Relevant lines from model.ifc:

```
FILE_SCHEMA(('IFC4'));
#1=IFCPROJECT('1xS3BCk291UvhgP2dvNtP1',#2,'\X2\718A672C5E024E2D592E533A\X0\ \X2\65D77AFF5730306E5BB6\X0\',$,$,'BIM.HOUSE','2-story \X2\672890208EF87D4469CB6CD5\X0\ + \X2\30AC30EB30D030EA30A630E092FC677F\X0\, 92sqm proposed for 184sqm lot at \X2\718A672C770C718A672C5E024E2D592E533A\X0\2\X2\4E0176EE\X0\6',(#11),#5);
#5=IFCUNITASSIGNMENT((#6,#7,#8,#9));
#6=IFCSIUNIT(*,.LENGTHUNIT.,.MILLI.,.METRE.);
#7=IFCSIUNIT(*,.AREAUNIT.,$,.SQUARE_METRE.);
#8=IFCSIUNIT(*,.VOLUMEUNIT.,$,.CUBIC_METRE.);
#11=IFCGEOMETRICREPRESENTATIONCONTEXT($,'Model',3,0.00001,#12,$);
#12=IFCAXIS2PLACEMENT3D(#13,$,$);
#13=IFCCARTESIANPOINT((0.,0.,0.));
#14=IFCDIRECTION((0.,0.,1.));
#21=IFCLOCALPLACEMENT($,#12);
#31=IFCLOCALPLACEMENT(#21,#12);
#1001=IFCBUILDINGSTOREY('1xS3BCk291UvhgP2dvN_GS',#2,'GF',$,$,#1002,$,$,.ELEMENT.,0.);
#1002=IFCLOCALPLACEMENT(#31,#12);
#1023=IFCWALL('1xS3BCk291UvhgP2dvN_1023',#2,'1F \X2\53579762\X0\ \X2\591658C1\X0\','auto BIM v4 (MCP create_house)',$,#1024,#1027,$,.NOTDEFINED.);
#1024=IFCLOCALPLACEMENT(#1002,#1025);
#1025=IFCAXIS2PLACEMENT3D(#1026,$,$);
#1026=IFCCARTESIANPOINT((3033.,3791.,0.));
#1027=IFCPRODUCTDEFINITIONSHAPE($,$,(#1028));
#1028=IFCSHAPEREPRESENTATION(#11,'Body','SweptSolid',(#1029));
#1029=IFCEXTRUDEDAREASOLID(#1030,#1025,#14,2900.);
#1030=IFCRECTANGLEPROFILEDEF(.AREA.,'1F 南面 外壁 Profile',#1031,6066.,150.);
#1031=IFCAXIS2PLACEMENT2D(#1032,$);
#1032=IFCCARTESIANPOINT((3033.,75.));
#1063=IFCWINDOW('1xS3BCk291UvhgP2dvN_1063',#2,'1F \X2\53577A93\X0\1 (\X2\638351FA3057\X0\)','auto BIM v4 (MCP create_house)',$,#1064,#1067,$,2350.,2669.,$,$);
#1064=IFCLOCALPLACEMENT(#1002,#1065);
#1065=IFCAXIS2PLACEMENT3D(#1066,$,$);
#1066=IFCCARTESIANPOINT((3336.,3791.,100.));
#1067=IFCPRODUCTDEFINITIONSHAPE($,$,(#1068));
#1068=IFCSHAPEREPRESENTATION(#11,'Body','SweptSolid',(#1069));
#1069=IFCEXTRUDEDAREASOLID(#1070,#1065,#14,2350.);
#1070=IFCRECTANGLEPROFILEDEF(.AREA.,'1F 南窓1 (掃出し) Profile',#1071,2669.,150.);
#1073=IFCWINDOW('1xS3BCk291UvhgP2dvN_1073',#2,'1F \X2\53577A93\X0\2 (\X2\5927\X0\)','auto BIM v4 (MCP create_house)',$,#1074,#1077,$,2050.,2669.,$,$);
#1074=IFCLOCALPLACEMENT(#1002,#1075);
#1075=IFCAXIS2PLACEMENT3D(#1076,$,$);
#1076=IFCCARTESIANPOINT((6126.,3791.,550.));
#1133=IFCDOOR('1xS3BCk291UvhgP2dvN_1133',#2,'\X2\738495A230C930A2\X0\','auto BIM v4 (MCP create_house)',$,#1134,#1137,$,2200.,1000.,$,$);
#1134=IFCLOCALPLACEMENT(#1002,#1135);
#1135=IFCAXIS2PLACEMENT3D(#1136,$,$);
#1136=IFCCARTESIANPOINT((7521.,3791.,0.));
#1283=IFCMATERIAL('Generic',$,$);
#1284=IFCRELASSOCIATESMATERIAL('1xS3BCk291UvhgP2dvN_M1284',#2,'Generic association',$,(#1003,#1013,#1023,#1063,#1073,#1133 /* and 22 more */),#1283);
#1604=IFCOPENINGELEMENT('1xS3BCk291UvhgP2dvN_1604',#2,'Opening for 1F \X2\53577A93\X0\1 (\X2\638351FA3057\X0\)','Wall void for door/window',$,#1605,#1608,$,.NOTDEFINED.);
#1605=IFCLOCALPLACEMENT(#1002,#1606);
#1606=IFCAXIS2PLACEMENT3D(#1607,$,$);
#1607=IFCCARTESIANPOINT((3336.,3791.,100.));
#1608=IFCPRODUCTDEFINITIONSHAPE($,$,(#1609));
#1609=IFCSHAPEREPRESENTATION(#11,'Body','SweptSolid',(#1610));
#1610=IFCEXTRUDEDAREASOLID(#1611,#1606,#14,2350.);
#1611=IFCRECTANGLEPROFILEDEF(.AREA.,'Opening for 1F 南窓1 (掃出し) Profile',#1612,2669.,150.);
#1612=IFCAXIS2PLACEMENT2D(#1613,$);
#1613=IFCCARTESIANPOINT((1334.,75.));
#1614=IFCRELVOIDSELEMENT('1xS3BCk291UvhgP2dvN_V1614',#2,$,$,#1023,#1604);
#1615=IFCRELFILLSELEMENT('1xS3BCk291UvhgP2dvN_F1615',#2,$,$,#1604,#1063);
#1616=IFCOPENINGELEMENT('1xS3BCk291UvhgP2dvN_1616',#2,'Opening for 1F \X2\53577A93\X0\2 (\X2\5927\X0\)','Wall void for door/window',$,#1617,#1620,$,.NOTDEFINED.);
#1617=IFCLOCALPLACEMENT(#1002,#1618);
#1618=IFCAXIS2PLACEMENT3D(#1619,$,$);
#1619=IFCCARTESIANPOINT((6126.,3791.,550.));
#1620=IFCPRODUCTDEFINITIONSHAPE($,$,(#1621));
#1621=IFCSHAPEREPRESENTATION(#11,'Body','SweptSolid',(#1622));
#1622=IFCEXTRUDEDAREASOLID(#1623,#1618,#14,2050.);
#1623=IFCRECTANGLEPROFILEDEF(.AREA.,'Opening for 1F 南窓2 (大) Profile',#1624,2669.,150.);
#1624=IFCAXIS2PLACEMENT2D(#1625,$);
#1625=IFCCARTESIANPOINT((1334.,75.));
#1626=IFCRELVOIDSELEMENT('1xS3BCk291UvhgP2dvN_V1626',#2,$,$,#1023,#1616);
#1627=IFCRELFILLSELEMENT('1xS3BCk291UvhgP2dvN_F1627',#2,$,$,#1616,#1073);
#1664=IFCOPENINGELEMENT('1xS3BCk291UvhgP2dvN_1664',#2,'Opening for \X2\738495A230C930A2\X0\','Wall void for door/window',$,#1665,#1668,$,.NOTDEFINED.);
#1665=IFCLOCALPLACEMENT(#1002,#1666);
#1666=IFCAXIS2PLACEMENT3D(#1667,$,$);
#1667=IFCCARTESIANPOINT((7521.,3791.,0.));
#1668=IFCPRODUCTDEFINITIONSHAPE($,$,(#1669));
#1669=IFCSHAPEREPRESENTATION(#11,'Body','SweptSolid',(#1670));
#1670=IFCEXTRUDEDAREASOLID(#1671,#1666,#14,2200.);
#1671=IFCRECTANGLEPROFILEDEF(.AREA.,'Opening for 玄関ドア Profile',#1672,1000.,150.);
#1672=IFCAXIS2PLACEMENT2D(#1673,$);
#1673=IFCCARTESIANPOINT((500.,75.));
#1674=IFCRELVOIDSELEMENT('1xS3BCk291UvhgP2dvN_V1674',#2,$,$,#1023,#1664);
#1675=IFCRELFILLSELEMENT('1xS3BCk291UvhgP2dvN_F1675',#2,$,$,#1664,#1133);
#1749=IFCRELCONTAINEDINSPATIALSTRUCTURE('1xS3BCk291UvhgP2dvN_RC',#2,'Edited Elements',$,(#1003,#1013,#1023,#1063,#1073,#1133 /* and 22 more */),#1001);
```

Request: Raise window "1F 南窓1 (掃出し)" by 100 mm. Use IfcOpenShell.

```python
import numpy as np
import ifcopenshell
import ifcopenshell.api.geometry
import ifcopenshell.util.placement
import ifcopenshell.util.unit

model = ifcopenshell.open("model.ifc")
unit_scale = ifcopenshell.util.unit.calculate_unit_scale(model)

window = model.by_guid("1xS3BCk291UvhgP2dvN_1063")
opening = window.FillsVoids[0].RelatingOpeningElement
dz = 0.1 / unit_scale

shift = np.array([0.0, 0.0, dz])
# The window is not placed relative to its opening, so move both.
for product in (opening, window):
    matrix = ifcopenshell.util.placement.get_local_placement(product.ObjectPlacement)
    matrix[:3, 3] += shift
    ifcopenshell.api.geometry.edit_object_placement(model, product=product, matrix=matrix, is_si=False)

print(f"moved by {dz * unit_scale:+.3f} m")

model.write("model_v2.ifc")
```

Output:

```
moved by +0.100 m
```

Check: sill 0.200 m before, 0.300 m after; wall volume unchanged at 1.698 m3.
